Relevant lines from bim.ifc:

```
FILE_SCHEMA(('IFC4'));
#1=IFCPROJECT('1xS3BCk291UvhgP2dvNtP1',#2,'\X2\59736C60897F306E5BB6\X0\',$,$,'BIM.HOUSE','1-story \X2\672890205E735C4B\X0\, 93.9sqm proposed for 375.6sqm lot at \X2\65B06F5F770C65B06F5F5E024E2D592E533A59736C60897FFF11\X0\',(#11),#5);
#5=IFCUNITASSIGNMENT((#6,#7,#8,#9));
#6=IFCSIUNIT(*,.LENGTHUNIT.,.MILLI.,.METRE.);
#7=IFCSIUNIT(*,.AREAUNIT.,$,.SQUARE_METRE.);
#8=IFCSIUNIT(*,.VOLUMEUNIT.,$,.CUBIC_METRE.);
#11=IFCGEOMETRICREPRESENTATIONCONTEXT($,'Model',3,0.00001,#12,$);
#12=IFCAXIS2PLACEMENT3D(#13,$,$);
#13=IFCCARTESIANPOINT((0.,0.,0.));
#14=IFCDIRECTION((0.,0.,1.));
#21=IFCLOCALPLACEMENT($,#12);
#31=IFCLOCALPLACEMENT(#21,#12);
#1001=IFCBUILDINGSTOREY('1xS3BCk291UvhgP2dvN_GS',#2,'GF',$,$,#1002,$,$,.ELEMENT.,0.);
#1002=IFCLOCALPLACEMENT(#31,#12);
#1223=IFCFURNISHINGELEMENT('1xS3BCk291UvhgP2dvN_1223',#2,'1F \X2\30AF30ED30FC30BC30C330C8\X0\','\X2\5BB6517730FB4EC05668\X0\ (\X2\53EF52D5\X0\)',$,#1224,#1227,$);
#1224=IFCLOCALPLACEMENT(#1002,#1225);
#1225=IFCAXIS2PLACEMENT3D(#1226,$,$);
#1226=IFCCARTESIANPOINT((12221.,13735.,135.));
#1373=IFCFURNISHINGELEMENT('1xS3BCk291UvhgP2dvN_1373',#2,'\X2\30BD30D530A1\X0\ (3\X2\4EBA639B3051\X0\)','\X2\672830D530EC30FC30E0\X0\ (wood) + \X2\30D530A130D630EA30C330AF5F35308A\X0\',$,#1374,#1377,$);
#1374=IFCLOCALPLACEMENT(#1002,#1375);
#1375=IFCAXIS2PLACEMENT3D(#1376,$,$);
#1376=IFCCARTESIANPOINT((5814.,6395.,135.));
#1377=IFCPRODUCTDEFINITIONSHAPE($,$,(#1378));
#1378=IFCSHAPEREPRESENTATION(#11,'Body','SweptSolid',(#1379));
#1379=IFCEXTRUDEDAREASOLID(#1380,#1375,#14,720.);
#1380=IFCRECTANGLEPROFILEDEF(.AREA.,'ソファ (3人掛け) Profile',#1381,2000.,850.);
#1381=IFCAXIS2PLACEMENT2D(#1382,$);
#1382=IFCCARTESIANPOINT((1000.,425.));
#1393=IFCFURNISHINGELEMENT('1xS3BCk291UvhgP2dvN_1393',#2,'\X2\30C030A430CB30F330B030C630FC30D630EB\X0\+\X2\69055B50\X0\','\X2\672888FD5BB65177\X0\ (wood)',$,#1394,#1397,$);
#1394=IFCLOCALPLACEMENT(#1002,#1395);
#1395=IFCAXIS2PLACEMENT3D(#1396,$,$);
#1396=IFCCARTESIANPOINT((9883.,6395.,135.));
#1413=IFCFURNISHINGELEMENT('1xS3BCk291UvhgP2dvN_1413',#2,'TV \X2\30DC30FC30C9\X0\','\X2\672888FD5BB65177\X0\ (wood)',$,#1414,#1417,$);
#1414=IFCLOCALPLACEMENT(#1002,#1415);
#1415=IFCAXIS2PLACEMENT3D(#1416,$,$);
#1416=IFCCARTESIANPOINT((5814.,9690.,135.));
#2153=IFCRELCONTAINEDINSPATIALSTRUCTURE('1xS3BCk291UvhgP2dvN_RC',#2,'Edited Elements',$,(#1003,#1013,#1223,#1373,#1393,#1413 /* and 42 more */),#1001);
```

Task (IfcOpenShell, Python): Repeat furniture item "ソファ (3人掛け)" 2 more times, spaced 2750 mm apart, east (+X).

```python
import numpy as np
import ifcopenshell
import ifcopenshell.api.geometry
import ifcopenshell.api.root
import ifcopenshell.util.element
import ifcopenshell.util.placement
import ifcopenshell.util.unit

model = ifcopenshell.open("bim.ifc")
unit_scale = ifcopenshell.util.unit.calculate_unit_scale(model)


def reuse_history(source, copy):
    """copy_class also copies each property set's owner history, people and application; keep the originals."""
    for rel in copy.IsDefinedBy:
        if rel.is_a("IfcRelDefinesByProperties") and (history := rel.RelatingPropertyDefinition.OwnerHistory):
            rel.RelatingPropertyDefinition.OwnerHistory = source.OwnerHistory
            ifcopenshell.util.element.remove_deep2(model, history)


source = model.by_guid("1xS3BCk291UvhgP2dvN_1373")
base = ifcopenshell.util.placement.get_local_placement(source.ObjectPlacement)
step = np.array([1.0, 0.0, 0.0]) * 2.75 / unit_scale

for i in range(1, 3):
    copy = ifcopenshell.api.root.copy_class(model, product=source)
    copy.Representation = ifcopenshell.util.element.copy_deep(
        model, source.Representation, exclude=["IfcGeometricRepresentationContext", "IfcRepresentationMap"]
    )
    reuse_history(source, copy)
    matrix = base.copy()
    matrix[:3, 3] += i * step
    print("added at", matrix[:3, 3].round(3) + 0.0)
    ifcopenshell.api.geometry.edit_object_placement(model, product=copy, matrix=matrix, is_si=False)

model.write("bim_edited.ifc")
```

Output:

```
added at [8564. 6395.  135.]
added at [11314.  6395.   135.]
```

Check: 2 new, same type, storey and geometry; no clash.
